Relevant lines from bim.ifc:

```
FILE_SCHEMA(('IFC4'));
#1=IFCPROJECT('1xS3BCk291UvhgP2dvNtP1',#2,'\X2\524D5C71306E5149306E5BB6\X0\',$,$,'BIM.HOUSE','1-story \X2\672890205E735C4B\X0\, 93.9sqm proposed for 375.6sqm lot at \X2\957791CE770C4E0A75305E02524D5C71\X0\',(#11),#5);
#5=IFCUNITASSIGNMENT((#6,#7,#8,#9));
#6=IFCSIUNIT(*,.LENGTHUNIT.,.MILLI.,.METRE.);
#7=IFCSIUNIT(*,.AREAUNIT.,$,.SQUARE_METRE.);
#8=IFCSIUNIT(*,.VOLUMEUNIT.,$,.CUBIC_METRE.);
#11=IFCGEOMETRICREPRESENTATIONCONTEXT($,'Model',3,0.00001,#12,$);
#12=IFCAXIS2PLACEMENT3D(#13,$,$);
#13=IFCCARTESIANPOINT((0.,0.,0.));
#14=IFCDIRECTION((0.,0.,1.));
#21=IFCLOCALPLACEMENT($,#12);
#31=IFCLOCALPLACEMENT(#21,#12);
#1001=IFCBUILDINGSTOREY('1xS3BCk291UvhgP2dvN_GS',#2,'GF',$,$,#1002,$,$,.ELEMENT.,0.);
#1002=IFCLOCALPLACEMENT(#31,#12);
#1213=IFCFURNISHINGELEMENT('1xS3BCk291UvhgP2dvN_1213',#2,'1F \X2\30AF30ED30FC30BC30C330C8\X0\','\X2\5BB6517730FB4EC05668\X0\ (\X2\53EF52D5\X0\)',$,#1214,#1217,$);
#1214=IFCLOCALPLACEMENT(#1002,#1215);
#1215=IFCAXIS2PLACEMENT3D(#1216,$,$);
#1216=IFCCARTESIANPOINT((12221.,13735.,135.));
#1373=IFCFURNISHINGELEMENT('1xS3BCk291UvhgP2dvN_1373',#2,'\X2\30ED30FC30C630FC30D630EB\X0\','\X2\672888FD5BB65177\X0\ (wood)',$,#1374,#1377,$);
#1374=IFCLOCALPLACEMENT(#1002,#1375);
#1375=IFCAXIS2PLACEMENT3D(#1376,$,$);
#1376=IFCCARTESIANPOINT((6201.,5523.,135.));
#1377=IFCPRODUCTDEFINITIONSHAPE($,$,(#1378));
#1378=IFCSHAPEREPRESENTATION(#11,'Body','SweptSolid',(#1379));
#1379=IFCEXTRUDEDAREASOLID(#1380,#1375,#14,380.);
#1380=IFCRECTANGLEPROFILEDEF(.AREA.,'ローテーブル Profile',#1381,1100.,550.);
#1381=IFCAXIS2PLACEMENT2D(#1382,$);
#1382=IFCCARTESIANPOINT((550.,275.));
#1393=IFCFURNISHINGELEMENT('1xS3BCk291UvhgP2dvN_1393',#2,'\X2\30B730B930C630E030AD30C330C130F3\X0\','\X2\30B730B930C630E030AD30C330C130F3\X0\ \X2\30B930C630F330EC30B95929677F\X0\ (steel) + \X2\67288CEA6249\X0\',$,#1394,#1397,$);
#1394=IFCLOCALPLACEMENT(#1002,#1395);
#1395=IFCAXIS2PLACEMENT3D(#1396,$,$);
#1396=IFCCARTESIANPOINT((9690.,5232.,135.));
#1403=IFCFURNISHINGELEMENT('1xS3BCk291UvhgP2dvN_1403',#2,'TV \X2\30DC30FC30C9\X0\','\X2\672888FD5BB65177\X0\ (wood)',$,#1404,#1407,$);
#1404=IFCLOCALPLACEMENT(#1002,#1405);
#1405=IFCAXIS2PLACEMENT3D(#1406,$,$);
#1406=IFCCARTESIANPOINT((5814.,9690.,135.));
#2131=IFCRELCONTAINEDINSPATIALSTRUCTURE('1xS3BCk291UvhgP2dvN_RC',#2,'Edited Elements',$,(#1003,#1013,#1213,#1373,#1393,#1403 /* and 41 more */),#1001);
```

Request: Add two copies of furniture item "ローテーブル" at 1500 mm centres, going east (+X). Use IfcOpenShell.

```python
import numpy as np
import ifcopenshell
import ifcopenshell.api.geometry
import ifcopenshell.api.root
import ifcopenshell.util.element
import ifcopenshell.util.placement
import ifcopenshell.util.unit

model = ifcopenshell.open("bim.ifc")
unit_scale = ifcopenshell.util.unit.calculate_unit_scale(model)


def reuse_history(source, copy):
    """copy_class also copies each property set's owner history, people and application; keep the originals."""
    for rel in copy.IsDefinedBy:
        if rel.is_a("IfcRelDefinesByProperties") and (history := rel.RelatingPropertyDefinition.OwnerHistory):
            rel.RelatingPropertyDefinition.OwnerHistory = source.OwnerHistory
            ifcopenshell.util.element.remove_deep2(model, history)


source = model.by_id(1373)
base = ifcopenshell.util.placement.get_local_placement(source.ObjectPlacement)
step = np.array([1.0, 0.0, 0.0]) * 1.5 / unit_scale

for i in range(1, 3):
    copy = ifcopenshell.api.root.copy_class(model, product=source)
    copy.Representation = ifcopenshell.util.element.copy_deep(
        model, source.Representation, exclude=["IfcGeometricRepresentationContext", "IfcRepresentationMap"]
    )
    reuse_history(source, copy)
    matrix = base.copy()
    matrix[:3, 3] += i * step
    print("added at", matrix[:3, 3].round(3) + 0.0)
    ifcopenshell.api.geometry.edit_object_placement(model, product=copy, matrix=matrix, is_si=False)

model.write("bim_v2.ifc")
```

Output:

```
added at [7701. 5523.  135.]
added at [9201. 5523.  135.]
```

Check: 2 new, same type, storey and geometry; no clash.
